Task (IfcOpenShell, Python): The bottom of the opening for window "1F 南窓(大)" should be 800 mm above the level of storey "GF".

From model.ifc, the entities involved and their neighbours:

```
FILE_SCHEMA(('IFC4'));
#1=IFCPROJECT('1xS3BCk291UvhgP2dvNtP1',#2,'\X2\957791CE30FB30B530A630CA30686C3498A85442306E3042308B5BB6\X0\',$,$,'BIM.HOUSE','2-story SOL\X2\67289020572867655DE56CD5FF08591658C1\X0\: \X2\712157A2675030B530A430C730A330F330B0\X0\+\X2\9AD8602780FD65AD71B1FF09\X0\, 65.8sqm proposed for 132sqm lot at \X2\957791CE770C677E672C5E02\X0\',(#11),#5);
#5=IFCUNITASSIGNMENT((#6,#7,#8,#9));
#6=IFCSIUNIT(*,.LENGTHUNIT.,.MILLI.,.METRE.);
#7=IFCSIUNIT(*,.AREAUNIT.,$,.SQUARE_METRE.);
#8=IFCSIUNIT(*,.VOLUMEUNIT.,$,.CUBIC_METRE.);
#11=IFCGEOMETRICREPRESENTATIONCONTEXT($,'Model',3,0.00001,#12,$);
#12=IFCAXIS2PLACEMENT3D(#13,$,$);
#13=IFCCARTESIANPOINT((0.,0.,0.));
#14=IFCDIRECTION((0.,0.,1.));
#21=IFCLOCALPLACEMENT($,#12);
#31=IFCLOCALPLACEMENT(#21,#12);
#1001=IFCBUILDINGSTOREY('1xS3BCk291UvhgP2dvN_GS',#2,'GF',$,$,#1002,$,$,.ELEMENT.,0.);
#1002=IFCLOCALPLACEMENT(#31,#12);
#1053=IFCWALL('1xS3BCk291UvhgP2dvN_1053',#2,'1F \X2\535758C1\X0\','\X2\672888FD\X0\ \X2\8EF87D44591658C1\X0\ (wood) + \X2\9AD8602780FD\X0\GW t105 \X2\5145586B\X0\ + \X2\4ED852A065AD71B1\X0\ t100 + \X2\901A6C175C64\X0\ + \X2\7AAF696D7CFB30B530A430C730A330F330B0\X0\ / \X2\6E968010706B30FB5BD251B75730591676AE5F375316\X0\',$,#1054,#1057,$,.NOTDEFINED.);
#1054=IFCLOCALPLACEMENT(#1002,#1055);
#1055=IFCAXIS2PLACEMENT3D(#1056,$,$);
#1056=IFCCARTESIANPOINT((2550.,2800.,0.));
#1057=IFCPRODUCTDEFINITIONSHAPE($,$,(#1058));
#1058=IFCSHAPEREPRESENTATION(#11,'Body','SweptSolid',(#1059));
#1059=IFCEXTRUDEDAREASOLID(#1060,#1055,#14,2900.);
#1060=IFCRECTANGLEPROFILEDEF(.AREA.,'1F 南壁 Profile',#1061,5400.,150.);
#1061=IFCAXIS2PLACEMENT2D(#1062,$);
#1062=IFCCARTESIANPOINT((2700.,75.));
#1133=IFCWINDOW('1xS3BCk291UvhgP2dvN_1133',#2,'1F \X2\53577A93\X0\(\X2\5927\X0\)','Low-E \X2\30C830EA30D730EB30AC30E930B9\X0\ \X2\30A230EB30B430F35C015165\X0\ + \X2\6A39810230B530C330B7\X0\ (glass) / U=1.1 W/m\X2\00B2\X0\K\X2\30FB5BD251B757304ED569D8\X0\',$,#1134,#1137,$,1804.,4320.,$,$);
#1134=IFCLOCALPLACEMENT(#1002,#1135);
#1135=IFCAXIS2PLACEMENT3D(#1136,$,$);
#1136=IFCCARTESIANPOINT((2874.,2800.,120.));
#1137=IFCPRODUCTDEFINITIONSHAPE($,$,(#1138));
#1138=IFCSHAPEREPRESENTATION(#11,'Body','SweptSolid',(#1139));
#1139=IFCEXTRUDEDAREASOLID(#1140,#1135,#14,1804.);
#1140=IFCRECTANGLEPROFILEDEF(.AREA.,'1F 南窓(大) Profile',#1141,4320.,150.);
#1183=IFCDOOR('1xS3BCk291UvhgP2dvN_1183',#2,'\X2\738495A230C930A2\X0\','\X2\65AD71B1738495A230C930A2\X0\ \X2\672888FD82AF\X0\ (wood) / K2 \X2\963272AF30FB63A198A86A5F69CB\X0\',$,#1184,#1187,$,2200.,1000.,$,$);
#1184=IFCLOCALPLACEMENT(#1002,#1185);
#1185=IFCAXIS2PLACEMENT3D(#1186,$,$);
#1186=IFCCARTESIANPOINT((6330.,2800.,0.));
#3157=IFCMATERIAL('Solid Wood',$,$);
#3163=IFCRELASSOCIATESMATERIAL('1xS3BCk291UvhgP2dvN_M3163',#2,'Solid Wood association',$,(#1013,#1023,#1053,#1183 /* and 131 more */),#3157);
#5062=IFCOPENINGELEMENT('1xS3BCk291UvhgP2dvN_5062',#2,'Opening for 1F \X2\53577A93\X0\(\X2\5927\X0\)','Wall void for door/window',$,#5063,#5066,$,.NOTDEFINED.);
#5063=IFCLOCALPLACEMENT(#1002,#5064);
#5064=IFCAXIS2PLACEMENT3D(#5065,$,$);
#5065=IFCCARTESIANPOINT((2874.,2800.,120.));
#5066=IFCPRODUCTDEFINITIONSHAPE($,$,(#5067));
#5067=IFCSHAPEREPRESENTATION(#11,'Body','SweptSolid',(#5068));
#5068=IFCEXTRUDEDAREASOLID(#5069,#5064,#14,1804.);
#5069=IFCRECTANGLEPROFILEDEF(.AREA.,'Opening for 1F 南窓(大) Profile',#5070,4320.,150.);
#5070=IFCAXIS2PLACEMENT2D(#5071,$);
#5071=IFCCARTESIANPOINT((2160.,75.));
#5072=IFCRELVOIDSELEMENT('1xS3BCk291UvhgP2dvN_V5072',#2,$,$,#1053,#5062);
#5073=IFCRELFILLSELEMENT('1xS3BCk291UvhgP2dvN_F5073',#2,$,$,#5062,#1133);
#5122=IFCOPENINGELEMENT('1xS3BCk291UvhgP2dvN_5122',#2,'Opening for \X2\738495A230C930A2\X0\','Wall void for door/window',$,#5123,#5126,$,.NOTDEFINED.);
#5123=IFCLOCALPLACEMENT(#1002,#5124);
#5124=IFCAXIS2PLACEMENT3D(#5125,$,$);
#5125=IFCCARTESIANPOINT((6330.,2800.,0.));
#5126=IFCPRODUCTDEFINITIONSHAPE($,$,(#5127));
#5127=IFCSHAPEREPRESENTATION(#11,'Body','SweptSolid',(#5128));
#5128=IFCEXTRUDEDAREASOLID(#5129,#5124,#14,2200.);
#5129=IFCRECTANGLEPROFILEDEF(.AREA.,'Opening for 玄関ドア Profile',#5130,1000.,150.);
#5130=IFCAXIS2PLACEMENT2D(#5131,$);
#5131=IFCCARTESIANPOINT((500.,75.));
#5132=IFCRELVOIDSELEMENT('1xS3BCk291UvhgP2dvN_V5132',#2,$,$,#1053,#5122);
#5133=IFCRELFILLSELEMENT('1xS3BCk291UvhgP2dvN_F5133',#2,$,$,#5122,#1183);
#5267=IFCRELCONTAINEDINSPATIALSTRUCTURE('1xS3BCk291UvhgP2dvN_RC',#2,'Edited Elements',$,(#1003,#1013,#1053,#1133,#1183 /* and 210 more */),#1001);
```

```python
import numpy as np
import ifcopenshell
import ifcopenshell.api.geometry
import ifcopenshell.geom
import ifcopenshell.util.element
import ifcopenshell.util.placement
import ifcopenshell.util.shape
import ifcopenshell.util.unit

model = ifcopenshell.open("model.ifc")
unit_scale = ifcopenshell.util.unit.calculate_unit_scale(model)

window = model.by_id(1133)
opening = window.FillsVoids[0].RelatingOpeningElement
storey = ifcopenshell.util.element.get_container(window, ifc_class="IfcBuildingStorey")
level = ifcopenshell.util.placement.get_local_placement(storey.ObjectPlacement)[2, 3]

# The opening's origin need not be at the sill, so measure its lowest point.
shape = ifcopenshell.geom.create_shape(ifcopenshell.geom.settings(), opening)
bottom = ifcopenshell.util.shape.get_shape_bottom_elevation(shape, shape.geometry) / unit_scale
dz = level + 0.8 / unit_scale - bottom

shift = np.array([0.0, 0.0, dz])
# The window is not placed relative to its opening, so move both.
for product in (opening, window):
    matrix = ifcopenshell.util.placement.get_local_placement(product.ObjectPlacement)
    matrix[:3, 3] += shift
    ifcopenshell.api.geometry.edit_object_placement(model, product=product, matrix=matrix, is_si=False)

print(f"moved by {dz * unit_scale:+.3f} m")

model.write("model_rev.ifc")
```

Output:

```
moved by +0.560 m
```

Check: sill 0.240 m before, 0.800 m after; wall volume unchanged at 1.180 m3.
